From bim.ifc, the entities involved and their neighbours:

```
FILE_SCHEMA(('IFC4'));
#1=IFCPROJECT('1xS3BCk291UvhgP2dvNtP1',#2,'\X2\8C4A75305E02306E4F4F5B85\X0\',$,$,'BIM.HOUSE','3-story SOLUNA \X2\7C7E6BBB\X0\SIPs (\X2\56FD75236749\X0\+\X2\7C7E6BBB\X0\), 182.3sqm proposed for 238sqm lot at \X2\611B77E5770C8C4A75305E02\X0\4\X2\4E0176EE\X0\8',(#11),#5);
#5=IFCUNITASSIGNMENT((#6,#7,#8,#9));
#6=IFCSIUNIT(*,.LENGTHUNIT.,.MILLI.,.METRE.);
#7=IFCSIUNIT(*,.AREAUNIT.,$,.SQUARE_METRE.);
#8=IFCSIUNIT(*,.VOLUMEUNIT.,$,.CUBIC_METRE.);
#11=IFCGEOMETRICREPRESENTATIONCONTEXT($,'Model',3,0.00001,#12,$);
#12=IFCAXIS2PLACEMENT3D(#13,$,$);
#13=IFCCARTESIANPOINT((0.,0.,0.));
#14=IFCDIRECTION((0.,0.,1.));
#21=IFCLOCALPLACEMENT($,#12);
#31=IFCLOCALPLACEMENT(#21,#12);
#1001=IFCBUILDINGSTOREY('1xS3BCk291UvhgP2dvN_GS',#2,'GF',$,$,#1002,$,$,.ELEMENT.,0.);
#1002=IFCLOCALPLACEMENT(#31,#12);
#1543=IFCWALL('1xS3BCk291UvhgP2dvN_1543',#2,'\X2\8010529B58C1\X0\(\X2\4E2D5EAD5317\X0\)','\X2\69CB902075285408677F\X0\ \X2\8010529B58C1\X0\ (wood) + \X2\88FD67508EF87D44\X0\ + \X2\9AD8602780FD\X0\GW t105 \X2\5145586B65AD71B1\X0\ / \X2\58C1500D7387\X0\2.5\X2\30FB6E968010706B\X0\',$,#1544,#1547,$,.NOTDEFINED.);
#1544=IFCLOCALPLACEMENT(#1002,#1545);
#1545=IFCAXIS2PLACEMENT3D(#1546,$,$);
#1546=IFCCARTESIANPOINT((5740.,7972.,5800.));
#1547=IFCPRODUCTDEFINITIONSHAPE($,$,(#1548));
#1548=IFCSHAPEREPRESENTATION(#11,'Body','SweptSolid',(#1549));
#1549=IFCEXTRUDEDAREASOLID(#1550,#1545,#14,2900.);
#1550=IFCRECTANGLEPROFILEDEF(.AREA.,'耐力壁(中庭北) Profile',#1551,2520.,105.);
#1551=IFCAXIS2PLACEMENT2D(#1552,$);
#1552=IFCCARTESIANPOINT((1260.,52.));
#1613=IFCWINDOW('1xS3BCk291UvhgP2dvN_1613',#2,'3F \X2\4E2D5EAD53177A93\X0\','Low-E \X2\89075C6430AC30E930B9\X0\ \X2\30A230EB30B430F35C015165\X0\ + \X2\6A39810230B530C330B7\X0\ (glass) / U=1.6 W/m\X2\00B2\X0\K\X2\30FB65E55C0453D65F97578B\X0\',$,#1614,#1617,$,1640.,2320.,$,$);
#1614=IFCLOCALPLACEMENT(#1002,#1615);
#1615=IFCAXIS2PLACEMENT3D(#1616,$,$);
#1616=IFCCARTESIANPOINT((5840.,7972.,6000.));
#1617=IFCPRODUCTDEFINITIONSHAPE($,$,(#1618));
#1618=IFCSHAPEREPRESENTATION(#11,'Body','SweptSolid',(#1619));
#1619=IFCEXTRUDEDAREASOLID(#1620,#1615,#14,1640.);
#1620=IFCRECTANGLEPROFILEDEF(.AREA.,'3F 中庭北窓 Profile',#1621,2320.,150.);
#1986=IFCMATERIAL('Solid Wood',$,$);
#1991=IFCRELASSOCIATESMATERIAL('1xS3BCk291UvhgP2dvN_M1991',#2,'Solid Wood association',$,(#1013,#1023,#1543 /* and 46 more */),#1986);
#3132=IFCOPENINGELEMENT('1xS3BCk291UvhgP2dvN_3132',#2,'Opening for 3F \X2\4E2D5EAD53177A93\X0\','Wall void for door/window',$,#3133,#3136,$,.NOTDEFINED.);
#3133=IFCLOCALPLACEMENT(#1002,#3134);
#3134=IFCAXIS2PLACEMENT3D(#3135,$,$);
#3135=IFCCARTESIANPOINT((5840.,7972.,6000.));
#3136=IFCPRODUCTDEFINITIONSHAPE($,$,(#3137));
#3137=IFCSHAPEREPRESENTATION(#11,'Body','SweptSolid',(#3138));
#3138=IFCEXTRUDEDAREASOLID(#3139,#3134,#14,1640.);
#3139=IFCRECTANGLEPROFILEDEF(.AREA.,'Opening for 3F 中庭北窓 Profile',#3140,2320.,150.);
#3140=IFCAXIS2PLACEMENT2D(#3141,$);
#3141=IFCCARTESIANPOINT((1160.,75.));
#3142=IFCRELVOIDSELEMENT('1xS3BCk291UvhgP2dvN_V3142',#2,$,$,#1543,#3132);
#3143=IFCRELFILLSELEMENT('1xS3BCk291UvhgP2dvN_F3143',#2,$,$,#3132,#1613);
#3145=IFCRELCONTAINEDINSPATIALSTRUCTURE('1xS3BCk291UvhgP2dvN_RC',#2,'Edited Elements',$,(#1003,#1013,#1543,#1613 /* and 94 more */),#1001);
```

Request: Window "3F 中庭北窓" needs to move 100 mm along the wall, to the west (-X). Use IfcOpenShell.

```python
import ifcopenshell
import ifcopenshell.api.geometry
import ifcopenshell.util.placement

model = ifcopenshell.open("bim.ifc")

window = model.by_guid("1xS3BCk291UvhgP2dvN_1613")
opening = window.FillsVoids[0].RelatingOpeningElement
wall = opening.VoidsElements[0].RelatingBuildingElement

wall_matrix = ifcopenshell.util.placement.get_local_placement(wall.ObjectPlacement)
shift = wall_matrix[:3, 0] * -100.0
before = ifcopenshell.util.placement.get_local_placement(window.ObjectPlacement)[:3, 3].copy()

# The window is not placed relative to its opening, so move both.
for product in (opening, window):
    matrix = ifcopenshell.util.placement.get_local_placement(product.ObjectPlacement)
    matrix[:3, 3] += shift
    ifcopenshell.api.geometry.edit_object_placement(model, product=product, matrix=matrix, is_si=False)

after = ifcopenshell.util.placement.get_local_placement(window.ObjectPlacement)[:3, 3]
print("window moved by", (after - before).round(3) + 0.0)

model.write("bim_v2.ifc")
```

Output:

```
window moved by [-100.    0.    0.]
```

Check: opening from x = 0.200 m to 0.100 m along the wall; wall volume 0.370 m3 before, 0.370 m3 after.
